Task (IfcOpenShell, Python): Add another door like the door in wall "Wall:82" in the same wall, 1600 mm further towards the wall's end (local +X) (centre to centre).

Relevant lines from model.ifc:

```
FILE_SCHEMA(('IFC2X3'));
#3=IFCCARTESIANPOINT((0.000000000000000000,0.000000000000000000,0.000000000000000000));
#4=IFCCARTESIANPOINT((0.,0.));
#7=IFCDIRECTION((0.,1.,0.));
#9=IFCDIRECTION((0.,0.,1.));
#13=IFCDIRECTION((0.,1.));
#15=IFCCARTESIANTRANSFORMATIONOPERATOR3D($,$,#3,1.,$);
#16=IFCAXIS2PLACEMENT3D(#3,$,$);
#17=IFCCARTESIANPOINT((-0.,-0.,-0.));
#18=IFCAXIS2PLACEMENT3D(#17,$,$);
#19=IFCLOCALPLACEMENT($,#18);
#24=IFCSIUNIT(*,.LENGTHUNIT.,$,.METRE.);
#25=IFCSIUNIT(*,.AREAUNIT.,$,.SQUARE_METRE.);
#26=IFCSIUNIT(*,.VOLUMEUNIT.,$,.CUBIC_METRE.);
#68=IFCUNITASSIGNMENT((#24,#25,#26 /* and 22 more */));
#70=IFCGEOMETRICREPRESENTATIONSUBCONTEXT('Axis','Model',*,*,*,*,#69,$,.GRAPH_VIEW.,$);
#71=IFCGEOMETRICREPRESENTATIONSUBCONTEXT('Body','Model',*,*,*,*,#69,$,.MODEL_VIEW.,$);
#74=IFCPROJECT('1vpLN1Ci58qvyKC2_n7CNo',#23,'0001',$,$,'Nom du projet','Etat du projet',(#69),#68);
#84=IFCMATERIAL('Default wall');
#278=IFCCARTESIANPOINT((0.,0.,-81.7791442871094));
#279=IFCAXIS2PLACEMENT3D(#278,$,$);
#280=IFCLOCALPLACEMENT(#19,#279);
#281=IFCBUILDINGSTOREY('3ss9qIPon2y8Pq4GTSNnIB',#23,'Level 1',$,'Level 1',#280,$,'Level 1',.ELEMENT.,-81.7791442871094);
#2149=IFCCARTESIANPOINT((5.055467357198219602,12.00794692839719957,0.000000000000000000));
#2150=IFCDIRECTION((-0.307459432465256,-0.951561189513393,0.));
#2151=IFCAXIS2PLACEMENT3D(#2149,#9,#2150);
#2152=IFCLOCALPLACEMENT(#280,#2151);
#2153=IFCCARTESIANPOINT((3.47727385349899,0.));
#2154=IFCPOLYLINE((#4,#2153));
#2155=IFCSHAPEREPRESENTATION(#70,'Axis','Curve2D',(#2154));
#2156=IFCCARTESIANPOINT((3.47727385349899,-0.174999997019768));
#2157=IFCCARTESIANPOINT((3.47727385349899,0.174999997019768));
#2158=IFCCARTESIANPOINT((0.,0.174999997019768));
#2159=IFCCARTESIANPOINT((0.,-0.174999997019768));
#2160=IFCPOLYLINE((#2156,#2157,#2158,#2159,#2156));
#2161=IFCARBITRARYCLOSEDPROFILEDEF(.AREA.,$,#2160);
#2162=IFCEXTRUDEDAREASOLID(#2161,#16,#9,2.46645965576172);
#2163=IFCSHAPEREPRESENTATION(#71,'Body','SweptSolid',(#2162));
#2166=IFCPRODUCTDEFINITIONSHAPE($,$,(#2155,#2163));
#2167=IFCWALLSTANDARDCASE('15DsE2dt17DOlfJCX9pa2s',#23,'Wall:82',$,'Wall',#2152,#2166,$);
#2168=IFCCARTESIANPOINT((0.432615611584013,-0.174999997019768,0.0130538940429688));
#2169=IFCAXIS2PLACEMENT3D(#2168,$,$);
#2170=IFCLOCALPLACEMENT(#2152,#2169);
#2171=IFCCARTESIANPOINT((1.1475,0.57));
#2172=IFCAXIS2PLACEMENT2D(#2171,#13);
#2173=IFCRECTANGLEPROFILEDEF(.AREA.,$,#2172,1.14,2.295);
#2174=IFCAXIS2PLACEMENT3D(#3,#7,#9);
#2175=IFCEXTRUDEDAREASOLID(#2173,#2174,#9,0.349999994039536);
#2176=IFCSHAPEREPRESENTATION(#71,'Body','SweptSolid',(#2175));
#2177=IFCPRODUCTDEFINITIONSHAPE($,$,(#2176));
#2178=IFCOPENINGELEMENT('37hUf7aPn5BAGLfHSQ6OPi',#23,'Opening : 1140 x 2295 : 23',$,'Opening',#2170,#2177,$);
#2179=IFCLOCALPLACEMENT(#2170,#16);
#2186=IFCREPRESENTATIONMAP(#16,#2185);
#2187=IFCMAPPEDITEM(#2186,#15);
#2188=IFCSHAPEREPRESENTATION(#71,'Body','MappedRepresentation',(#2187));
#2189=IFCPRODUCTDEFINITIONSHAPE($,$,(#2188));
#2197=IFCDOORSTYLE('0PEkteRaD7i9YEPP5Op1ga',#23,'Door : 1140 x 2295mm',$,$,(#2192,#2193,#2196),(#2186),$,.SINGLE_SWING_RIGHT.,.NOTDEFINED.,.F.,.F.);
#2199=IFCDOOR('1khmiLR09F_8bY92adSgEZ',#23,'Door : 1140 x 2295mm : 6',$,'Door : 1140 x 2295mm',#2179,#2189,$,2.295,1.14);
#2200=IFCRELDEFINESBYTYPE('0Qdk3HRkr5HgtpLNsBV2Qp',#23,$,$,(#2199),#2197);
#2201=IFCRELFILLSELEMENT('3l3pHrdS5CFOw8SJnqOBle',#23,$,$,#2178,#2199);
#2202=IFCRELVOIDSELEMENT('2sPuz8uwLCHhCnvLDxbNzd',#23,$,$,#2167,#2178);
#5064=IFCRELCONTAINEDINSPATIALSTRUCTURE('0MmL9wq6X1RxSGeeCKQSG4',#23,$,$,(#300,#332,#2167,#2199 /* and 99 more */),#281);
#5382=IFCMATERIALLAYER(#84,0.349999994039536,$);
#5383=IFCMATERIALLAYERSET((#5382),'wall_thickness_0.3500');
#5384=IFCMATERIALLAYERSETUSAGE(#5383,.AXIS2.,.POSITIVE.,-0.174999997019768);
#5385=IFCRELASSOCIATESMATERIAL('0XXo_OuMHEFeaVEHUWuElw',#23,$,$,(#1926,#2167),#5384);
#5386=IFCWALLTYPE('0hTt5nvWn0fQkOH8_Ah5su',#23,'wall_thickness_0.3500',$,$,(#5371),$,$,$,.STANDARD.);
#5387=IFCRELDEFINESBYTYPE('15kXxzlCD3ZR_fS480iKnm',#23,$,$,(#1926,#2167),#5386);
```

```python
import ifcopenshell
import ifcopenshell.api.feature
import ifcopenshell.api.geometry
import ifcopenshell.api.root
import ifcopenshell.geom
import ifcopenshell.util.element
import ifcopenshell.util.placement
import ifcopenshell.util.shape

model = ifcopenshell.open("model.ifc")
settings = ifcopenshell.geom.settings()


def volume(element):
    """Net volume in cubic metres, openings subtracted."""
    shape = ifcopenshell.geom.create_shape(settings, element)
    return ifcopenshell.util.shape.get_volume(shape.geometry)


door = model.by_id(2199)
opening = door.FillsVoids[0].RelatingOpeningElement
wall = opening.VoidsElements[0].RelatingBuildingElement
before = volume(wall)
shift = ifcopenshell.util.placement.get_local_placement(wall.ObjectPlacement)[:3, 0] * 1.6

# copy_class copies the void relationship, type, container and properties, but no geometry.
new_opening = ifcopenshell.api.root.copy_class(model, product=opening)
new_opening.Representation = ifcopenshell.util.element.copy_deep(
    model, opening.Representation, exclude=["IfcGeometricRepresentationContext", "IfcRepresentationMap"]
)
new_opening.Name = "Opening : 1140 x 2295"
new_door = ifcopenshell.api.root.copy_class(model, product=door)
new_door.Representation = ifcopenshell.util.element.copy_deep(
    model, door.Representation, exclude=["IfcGeometricRepresentationContext", "IfcRepresentationMap"]
)
new_door.Name = "Door : 1140 x 2295mm"
fills = ifcopenshell.api.feature.add_filling(model, opening=new_opening, element=new_door)
fills.OwnerHistory = new_door.OwnerHistory  # required in IFC2X3

for old, new in ((opening, new_opening), (door, new_door)):
    matrix = ifcopenshell.util.placement.get_local_placement(old.ObjectPlacement)
    matrix[:3, 3] += shift
    ifcopenshell.api.geometry.edit_object_placement(model, product=new, matrix=matrix, is_si=False)

after = volume(wall)

print(f"wall volume {before:.3f} -> {after:.3f} m3")

model.write("model-out.ifc")
```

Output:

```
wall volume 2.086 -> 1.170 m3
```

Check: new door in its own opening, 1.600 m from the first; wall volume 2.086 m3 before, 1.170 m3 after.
